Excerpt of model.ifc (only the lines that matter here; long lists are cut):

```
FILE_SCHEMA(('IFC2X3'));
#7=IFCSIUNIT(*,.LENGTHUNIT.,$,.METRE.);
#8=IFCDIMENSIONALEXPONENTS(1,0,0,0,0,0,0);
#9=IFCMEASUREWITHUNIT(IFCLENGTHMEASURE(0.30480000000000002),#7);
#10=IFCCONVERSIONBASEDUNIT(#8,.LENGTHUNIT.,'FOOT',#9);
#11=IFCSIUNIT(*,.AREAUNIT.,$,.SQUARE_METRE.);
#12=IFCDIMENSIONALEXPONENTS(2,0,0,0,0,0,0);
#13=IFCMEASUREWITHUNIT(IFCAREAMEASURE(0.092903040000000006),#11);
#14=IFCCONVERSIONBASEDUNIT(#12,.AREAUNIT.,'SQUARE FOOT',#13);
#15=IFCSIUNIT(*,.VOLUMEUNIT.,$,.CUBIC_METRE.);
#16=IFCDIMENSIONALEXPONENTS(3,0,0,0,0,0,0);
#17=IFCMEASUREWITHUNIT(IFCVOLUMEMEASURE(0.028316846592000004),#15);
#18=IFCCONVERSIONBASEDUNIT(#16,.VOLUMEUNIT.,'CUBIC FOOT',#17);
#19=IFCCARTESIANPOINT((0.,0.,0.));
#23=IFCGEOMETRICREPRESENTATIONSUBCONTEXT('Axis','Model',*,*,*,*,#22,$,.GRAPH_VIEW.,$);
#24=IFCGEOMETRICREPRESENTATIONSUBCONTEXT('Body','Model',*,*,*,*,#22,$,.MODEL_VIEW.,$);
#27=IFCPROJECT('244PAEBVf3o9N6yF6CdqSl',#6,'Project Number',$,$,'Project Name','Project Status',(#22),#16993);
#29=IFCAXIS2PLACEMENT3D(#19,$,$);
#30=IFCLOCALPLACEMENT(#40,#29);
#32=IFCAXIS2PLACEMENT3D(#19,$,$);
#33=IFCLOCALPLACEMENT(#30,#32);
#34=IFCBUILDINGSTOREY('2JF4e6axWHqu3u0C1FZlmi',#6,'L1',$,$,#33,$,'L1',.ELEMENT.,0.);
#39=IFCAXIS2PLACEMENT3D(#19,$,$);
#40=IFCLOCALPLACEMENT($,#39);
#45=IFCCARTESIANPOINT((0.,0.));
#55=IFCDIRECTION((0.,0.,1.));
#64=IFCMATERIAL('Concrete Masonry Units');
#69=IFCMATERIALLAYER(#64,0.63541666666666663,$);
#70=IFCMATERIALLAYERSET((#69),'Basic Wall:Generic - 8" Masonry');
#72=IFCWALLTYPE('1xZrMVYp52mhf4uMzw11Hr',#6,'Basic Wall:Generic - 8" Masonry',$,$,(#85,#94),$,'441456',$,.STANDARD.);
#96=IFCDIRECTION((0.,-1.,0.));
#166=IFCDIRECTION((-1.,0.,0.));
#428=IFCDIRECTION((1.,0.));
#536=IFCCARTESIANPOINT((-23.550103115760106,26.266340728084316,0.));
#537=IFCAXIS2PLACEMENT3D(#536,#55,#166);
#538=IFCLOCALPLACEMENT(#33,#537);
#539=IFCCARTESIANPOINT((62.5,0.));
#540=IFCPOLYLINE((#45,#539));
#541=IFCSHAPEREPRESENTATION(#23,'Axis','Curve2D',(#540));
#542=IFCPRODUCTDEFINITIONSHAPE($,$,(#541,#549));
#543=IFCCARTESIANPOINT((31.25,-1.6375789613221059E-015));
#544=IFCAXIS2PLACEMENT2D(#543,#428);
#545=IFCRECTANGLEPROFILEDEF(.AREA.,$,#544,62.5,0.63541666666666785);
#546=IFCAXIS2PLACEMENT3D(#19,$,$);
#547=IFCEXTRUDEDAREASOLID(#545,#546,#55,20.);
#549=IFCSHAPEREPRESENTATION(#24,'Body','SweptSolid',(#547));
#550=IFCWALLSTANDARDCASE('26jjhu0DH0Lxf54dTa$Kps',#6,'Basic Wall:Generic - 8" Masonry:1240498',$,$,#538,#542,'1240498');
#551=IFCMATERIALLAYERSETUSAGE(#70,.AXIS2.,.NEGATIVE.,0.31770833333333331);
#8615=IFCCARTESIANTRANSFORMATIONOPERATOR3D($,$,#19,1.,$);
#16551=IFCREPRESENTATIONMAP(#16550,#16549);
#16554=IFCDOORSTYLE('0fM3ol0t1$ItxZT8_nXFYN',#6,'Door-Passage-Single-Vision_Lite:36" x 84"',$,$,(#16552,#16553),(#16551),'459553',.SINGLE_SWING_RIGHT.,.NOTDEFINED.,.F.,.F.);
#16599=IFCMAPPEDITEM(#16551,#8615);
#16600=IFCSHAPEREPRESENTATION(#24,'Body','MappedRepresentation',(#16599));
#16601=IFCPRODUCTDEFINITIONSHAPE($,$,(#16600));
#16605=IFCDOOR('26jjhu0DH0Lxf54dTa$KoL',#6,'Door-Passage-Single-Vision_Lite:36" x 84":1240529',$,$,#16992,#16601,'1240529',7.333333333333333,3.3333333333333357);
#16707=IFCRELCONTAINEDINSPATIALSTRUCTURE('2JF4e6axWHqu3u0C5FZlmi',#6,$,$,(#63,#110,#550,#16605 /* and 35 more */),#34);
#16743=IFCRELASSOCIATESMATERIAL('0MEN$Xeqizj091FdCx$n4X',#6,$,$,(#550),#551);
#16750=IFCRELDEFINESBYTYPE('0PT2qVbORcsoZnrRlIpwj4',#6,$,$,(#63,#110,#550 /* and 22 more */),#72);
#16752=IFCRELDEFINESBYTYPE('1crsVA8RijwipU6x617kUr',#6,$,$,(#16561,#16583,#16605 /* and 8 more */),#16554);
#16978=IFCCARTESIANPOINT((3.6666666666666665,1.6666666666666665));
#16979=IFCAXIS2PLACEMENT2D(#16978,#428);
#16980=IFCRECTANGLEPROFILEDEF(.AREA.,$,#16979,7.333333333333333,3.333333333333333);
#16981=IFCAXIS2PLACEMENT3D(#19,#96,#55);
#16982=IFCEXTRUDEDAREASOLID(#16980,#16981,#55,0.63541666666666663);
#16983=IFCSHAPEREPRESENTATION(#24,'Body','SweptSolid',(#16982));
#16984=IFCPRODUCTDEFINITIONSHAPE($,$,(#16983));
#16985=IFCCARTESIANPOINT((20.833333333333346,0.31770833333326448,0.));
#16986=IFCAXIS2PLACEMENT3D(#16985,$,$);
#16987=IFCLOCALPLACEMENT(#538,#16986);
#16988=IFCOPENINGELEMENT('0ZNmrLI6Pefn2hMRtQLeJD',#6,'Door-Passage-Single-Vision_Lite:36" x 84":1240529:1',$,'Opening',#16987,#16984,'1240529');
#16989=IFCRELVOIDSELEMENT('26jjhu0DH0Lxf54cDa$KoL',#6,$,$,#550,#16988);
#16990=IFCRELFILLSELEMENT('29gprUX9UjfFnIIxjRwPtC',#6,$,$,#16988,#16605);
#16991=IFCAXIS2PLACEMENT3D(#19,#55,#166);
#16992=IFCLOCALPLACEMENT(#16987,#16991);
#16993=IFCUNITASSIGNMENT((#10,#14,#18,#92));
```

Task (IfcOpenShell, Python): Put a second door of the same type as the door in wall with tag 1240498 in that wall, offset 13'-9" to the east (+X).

```python
import ifcopenshell
import ifcopenshell.api.feature
import ifcopenshell.api.geometry
import ifcopenshell.api.root
import ifcopenshell.geom
import ifcopenshell.util.element
import ifcopenshell.util.placement
import ifcopenshell.util.shape
import ifcopenshell.util.unit

model = ifcopenshell.open("model.ifc")
unit_scale = ifcopenshell.util.unit.calculate_unit_scale(model)
settings = ifcopenshell.geom.settings()


def volume(element):
    """Net volume in cubic metres, openings subtracted."""
    shape = ifcopenshell.geom.create_shape(settings, element)
    return ifcopenshell.util.shape.get_volume(shape.geometry)


def reuse_history(source, copy):
    """copy_class also copies each property set's owner history, people and application; keep the originals."""
    for rel in copy.IsDefinedBy:
        if rel.is_a("IfcRelDefinesByProperties") and (history := rel.RelatingPropertyDefinition.OwnerHistory):
            rel.RelatingPropertyDefinition.OwnerHistory = source.OwnerHistory
            ifcopenshell.util.element.remove_deep2(model, history)


door = model.by_guid("26jjhu0DH0Lxf54dTa$KoL")
opening = door.FillsVoids[0].RelatingOpeningElement
wall = opening.VoidsElements[0].RelatingBuildingElement
before = volume(wall)
shift = ifcopenshell.util.placement.get_local_placement(wall.ObjectPlacement)[:3, 0] * -165 * 0.0254 / unit_scale

# copy_class copies the void relationship, type, container and properties, but no geometry.
new_opening = ifcopenshell.api.root.copy_class(model, product=opening)
new_opening.Representation = ifcopenshell.util.element.copy_deep(
    model, opening.Representation, exclude=["IfcGeometricRepresentationContext", "IfcRepresentationMap"]
)
new_opening.Name = 'Door-Passage-Single-Vision_Lite:36" x 84"'
new_opening.Tag = None
new_door = ifcopenshell.api.root.copy_class(model, product=door)
new_door.Representation = ifcopenshell.util.element.copy_deep(
    model, door.Representation, exclude=["IfcGeometricRepresentationContext", "IfcRepresentationMap"]
)
new_door.Name = 'Door-Passage-Single-Vision_Lite:36" x 84"'
new_door.Tag = None
reuse_history(door, new_door)
fills = ifcopenshell.api.feature.add_filling(model, opening=new_opening, element=new_door)
fills.OwnerHistory = new_door.OwnerHistory  # required in IFC2X3

for old, new in ((opening, new_opening), (door, new_door)):
    matrix = ifcopenshell.util.placement.get_local_placement(old.ObjectPlacement)
    matrix[:3, 3] += shift
    ifcopenshell.api.geometry.edit_object_placement(model, product=new, matrix=matrix, is_si=False)

after = volume(wall)

print(f"wall volume {before:.3f} -> {after:.3f} m3")

model.write("model_v2.ifc")
```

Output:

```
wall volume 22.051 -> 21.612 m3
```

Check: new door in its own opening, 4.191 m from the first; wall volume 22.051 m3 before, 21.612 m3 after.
